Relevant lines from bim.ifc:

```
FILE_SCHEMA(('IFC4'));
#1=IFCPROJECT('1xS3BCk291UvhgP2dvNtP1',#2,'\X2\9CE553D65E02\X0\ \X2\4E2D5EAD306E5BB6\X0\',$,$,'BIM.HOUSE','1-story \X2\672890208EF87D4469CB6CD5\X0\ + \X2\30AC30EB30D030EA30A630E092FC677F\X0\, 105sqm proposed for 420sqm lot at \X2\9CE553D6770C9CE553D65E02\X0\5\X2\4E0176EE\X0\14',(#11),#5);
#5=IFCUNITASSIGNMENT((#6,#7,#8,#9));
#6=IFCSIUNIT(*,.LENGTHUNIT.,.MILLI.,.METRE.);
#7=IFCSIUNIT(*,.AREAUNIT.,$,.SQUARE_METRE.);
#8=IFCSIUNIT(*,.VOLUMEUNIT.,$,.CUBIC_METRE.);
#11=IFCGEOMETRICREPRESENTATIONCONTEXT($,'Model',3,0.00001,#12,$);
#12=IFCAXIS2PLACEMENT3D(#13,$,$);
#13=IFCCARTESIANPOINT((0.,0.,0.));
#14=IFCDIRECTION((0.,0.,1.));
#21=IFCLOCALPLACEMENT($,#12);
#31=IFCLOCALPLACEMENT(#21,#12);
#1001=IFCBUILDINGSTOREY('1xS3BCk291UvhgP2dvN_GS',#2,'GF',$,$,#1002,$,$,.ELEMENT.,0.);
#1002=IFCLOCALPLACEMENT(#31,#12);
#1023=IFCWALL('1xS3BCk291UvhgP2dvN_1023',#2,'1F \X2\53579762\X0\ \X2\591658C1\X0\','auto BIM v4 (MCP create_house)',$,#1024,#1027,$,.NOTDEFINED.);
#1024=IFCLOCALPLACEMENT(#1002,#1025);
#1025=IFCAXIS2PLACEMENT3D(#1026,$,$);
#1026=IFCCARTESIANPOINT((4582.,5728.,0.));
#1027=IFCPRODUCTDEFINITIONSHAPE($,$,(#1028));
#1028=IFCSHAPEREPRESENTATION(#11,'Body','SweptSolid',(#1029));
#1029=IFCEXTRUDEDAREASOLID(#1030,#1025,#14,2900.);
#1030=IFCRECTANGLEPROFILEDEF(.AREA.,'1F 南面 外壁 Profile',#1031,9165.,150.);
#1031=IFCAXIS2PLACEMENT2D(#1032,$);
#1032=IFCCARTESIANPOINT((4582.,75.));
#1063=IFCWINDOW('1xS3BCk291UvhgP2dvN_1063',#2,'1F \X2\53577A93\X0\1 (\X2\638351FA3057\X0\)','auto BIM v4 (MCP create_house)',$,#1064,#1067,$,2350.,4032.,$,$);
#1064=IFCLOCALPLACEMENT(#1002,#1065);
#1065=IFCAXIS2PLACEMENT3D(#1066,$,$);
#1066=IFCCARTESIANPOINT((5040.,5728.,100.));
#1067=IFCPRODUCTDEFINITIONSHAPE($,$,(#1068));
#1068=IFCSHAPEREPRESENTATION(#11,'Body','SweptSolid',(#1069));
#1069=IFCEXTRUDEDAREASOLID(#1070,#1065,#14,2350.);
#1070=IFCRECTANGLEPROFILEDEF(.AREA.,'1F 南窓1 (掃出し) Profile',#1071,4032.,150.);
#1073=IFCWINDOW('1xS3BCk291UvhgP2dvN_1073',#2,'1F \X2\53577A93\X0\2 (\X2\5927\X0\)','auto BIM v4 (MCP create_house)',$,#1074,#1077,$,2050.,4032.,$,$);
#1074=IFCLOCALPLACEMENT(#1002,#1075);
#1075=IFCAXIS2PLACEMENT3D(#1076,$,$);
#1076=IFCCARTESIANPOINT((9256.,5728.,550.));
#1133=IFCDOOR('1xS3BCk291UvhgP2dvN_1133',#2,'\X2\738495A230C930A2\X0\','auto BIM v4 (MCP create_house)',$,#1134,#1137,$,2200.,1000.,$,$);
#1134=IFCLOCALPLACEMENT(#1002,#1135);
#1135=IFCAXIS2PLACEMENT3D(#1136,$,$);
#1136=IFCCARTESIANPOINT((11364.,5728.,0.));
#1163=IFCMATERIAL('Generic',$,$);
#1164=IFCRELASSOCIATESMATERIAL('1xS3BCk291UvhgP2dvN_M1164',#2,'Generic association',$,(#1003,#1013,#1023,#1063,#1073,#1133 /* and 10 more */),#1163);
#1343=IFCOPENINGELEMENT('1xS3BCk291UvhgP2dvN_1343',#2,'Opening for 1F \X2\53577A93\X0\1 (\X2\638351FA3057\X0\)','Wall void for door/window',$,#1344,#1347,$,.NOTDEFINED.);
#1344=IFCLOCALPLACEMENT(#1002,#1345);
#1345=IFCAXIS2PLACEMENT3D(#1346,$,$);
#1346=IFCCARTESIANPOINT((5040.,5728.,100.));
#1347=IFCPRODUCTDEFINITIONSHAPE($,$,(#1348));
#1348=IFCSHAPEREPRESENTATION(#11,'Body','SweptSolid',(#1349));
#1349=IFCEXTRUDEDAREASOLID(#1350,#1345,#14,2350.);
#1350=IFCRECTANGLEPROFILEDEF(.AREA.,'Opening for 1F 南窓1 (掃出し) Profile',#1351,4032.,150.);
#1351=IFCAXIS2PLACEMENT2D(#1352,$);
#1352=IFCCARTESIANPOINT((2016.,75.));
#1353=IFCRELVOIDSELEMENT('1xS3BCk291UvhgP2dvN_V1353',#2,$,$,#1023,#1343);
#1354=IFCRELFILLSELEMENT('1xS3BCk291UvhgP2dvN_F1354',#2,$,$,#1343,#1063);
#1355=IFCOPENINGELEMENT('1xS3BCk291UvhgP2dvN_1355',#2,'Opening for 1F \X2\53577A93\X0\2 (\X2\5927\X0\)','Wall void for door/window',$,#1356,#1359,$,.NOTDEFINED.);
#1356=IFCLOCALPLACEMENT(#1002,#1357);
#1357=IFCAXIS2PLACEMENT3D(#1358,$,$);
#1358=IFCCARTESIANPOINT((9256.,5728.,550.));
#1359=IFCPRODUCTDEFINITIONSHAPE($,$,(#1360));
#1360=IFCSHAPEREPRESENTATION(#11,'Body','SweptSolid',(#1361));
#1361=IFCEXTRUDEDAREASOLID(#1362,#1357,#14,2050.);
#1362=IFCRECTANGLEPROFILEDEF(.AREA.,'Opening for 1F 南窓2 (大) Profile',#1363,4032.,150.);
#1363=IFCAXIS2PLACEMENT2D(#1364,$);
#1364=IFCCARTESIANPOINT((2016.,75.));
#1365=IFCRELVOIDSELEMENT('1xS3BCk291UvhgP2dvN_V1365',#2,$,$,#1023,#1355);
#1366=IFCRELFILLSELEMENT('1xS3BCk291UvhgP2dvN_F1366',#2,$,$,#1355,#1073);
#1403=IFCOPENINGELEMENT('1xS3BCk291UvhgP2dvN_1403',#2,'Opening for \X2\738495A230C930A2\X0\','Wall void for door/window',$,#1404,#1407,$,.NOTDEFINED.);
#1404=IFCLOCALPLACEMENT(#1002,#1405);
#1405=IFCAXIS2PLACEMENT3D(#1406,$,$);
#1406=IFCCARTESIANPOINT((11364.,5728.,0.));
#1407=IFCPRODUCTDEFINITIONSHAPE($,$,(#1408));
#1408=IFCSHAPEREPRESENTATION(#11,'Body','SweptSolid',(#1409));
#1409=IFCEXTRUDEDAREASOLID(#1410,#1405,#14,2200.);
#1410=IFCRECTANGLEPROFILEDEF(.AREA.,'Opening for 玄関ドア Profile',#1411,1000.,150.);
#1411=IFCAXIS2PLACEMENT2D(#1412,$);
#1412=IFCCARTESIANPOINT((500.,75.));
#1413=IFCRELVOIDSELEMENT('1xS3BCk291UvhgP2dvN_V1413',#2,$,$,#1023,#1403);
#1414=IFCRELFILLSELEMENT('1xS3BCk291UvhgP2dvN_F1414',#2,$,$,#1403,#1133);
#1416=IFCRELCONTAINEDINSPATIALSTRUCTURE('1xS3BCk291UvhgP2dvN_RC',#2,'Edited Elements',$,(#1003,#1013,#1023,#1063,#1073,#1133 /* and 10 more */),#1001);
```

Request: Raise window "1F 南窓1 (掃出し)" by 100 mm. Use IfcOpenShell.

```python
import numpy as np
import ifcopenshell
import ifcopenshell.api.geometry
import ifcopenshell.util.placement
import ifcopenshell.util.unit

model = ifcopenshell.open("bim.ifc")
unit_scale = ifcopenshell.util.unit.calculate_unit_scale(model)

window = model.by_guid("1xS3BCk291UvhgP2dvN_1063")
opening = window.FillsVoids[0].RelatingOpeningElement
dz = 100.0

shift = np.array([0.0, 0.0, dz])
# The window is not placed relative to its opening, so move both.
for product in (opening, window):
    matrix = ifcopenshell.util.placement.get_local_placement(product.ObjectPlacement)
    matrix[:3, 3] += shift
    ifcopenshell.api.geometry.edit_object_placement(model, product=product, matrix=matrix, is_si=False)

print(f"moved by {dz * unit_scale:+.3f} m")

model.write("bim-out.ifc")
```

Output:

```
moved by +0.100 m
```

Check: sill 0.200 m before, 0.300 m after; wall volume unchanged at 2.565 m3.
